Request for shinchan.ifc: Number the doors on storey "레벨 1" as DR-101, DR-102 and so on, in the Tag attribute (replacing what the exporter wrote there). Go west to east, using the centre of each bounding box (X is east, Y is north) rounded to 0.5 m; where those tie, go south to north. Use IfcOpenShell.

First a look at what the model holds.

```python
import ifcopenshell
import ifcopenshell.util.element
import ifcopenshell.util.placement

model = ifcopenshell.open("shinchan.ifc")
print(model.schema)
storey = next(s for s in model.by_type("IfcBuildingStorey") if s.Name == "레벨 1")
doors = [e for e in ifcopenshell.util.element.get_decomposition(storey) if e.is_a("IfcDoor")]
for e in sorted(doors, key=lambda e: e.id()):
    origin = ifcopenshell.util.placement.get_local_placement(e.ObjectPlacement)[:3, 3]
    print(e.id(), e.Tag, e.Name, origin.round(2) + 0.0, sep=" | ")
```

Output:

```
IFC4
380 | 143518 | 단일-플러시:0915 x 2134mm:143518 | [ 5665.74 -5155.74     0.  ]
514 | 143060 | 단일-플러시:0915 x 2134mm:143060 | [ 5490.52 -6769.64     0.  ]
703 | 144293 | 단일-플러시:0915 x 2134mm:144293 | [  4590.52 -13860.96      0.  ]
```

```python
import ifcopenshell
import ifcopenshell.geom
import ifcopenshell.util.element
import ifcopenshell.util.shape

model = ifcopenshell.open("shinchan.ifc")
settings = ifcopenshell.geom.settings()
settings.set("use-world-coords", True)


def centre(element):
    shape = ifcopenshell.geom.create_shape(settings, element)
    return ifcopenshell.util.shape.get_bbox_centroid(shape.geometry)


storey = next(s for s in model.by_type("IfcBuildingStorey") if s.Name == "레벨 1")
doors = [e for e in ifcopenshell.util.element.get_decomposition(storey) if e.is_a("IfcDoor")]

# Insertion points can sit at a corner or the storey origin, so sort by the geometry (in metres).
centres = {e: centre(e) for e in doors}
doors.sort(key=lambda e: (round(centres[e][0] / 0.5), centres[e][1]))

for i, e in enumerate(doors, start=1):
    number = f"DR-1{i:02d}"
    e.Tag = number
    print(e.id(), number)

model.write("shinchan_v2.ifc")
```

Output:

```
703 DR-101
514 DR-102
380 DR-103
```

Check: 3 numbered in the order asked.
